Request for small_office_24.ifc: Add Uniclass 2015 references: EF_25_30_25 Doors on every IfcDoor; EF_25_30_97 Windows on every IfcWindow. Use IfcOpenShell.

First a look at what the model holds.

```python
import ifcopenshell

model = ifcopenshell.open("small_office_24.ifc")
print(model.schema)
print("classifications:", [c.Name for c in model.by_type("IfcClassification")])
for ifc_class in ("IfcDoor", "IfcRoof", "IfcStair", "IfcWall", "IfcWindow"):
    print(ifc_class, len(model.by_type(ifc_class)))
```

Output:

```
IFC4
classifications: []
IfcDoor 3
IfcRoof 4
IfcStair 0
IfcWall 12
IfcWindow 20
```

```python
import ifcopenshell
import ifcopenshell.api.classification

model = ifcopenshell.open("small_office_24.ifc")

system = ifcopenshell.api.classification.add_classification(model, classification="Uniclass 2015")

codes = {
    "IfcDoor": ("EF_25_30_25", "Doors"),
    "IfcWindow": ("EF_25_30_97", "Windows"),
}
for ifc_class, (code, name) in codes.items():
    products = model.by_type(ifc_class)
    ifcopenshell.api.classification.add_reference(
        model, products=products, classification=system, identification=code, name=name
    )
    print(code, len(products))

model.write("small_office_24_rev.ifc")
```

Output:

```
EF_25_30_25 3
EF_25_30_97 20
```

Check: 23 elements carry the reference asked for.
